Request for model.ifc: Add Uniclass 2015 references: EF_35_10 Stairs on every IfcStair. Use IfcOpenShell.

First a look at what the model holds.

```python
import ifcopenshell

model = ifcopenshell.open("model.ifc")
print(model.schema)
print("classifications:", [c.Name for c in model.by_type("IfcClassification")])
for ifc_class in ("IfcDoor", "IfcRoof", "IfcStair", "IfcWall", "IfcWindow"):
    print(ifc_class, len(model.by_type(ifc_class)))
```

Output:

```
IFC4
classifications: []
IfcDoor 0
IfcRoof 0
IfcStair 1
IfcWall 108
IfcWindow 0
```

```python
import ifcopenshell
import ifcopenshell.api.classification

model = ifcopenshell.open("model.ifc")

system = ifcopenshell.api.classification.add_classification(model, classification="Uniclass 2015")

codes = {
    "IfcStair": ("EF_35_10", "Stairs"),
}
for ifc_class, (code, name) in codes.items():
    products = model.by_type(ifc_class)
    ifcopenshell.api.classification.add_reference(
        model, products=products, classification=system, identification=code, name=name
    )
    print(code, len(products))

model.write("model-out.ifc")
```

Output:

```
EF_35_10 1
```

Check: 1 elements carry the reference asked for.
